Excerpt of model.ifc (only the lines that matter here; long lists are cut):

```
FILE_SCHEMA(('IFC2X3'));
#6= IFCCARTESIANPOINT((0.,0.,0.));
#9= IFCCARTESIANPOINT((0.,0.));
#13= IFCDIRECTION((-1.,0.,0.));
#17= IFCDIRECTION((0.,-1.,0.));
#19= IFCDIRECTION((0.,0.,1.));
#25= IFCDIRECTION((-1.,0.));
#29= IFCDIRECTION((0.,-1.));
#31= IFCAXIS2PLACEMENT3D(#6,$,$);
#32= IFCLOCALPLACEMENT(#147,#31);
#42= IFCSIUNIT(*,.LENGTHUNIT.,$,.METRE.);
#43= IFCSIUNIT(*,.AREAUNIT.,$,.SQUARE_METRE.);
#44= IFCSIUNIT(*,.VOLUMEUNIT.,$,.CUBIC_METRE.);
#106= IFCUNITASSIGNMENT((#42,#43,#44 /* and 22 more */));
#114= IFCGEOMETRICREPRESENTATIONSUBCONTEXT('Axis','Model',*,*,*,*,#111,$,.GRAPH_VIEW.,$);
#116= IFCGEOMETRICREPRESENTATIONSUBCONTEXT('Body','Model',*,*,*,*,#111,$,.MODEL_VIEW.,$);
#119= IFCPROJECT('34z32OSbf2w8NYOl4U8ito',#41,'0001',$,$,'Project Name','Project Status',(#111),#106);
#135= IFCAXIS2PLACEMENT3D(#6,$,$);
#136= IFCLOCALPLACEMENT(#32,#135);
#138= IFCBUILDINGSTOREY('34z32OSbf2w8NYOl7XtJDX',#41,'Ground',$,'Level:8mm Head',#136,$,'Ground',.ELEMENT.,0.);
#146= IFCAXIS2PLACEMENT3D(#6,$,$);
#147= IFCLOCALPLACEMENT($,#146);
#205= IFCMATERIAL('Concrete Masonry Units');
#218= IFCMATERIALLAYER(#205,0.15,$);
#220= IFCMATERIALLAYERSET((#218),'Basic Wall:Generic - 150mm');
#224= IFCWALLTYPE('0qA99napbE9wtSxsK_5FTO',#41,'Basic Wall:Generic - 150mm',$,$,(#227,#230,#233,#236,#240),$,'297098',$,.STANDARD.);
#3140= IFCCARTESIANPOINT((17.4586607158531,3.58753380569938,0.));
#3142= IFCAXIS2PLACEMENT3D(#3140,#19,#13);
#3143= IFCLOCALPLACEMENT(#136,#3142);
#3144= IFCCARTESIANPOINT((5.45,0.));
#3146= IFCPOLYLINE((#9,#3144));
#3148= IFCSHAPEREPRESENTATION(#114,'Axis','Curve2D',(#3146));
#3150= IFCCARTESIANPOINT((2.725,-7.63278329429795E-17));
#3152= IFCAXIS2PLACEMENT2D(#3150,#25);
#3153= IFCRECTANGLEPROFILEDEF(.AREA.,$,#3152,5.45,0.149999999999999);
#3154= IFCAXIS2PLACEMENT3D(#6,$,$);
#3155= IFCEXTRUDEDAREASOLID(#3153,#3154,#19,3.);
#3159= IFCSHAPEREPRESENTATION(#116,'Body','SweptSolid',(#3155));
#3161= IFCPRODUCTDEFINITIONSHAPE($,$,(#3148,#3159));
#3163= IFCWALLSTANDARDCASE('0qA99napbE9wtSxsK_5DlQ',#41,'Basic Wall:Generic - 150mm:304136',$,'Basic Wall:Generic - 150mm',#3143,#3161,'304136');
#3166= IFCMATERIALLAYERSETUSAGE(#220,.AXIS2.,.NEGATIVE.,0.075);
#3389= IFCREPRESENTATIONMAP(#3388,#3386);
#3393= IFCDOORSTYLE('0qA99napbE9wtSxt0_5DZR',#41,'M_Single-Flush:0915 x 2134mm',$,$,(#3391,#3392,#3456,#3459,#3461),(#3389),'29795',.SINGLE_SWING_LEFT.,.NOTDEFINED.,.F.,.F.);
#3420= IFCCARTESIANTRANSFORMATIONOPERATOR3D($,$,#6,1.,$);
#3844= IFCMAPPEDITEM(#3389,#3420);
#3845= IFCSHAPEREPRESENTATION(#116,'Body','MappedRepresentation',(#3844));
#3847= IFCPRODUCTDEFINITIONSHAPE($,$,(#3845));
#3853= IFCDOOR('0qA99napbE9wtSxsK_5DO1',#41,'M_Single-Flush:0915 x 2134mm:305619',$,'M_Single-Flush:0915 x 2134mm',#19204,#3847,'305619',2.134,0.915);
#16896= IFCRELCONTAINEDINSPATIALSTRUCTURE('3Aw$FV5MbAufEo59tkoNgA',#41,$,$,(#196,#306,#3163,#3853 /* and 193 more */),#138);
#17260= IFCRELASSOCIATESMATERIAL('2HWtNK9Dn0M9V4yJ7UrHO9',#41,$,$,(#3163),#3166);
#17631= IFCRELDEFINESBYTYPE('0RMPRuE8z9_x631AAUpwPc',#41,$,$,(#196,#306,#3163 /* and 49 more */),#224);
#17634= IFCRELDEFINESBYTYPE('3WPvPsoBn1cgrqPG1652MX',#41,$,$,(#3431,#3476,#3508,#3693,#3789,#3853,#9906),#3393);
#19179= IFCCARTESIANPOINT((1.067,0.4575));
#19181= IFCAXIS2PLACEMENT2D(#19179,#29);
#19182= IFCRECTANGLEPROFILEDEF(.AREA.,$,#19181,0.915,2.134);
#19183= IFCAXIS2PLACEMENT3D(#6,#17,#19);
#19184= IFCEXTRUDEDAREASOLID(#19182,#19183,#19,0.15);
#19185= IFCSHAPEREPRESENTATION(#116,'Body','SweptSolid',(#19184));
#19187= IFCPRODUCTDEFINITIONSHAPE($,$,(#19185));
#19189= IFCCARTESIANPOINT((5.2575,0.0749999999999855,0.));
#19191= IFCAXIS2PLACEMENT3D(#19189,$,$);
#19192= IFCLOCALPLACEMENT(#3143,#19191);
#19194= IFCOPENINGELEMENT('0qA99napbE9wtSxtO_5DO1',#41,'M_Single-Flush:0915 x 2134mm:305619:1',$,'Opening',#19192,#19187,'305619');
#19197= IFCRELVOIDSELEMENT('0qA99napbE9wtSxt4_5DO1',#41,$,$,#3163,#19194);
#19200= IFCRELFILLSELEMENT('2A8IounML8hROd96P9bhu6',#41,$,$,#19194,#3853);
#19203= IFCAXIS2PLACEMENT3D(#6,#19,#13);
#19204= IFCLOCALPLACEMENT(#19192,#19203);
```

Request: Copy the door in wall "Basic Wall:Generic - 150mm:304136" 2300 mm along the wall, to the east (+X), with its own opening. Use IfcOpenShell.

```python
import ifcopenshell
import ifcopenshell.api.feature
import ifcopenshell.api.geometry
import ifcopenshell.api.root
import ifcopenshell.geom
import ifcopenshell.util.element
import ifcopenshell.util.placement
import ifcopenshell.util.shape

model = ifcopenshell.open("model.ifc")
settings = ifcopenshell.geom.settings()


def volume(element):
    """Net volume in cubic metres, openings subtracted."""
    shape = ifcopenshell.geom.create_shape(settings, element)
    return ifcopenshell.util.shape.get_volume(shape.geometry)


def reuse_history(source, copy):
    """copy_class also copies each property set's owner history, people and application; keep the originals."""
    for rel in copy.IsDefinedBy:
        if rel.is_a("IfcRelDefinesByProperties") and (history := rel.RelatingPropertyDefinition.OwnerHistory):
            rel.RelatingPropertyDefinition.OwnerHistory = source.OwnerHistory
            ifcopenshell.util.element.remove_deep2(model, history)


door = model.by_guid("0qA99napbE9wtSxsK_5DO1")
opening = door.FillsVoids[0].RelatingOpeningElement
wall = opening.VoidsElements[0].RelatingBuildingElement
before = volume(wall)
shift = ifcopenshell.util.placement.get_local_placement(wall.ObjectPlacement)[:3, 0] * -2.3

# copy_class copies the void relationship, type, container and properties, but no geometry.
new_opening = ifcopenshell.api.root.copy_class(model, product=opening)
new_opening.Representation = ifcopenshell.util.element.copy_deep(
    model, opening.Representation, exclude=["IfcGeometricRepresentationContext", "IfcRepresentationMap"]
)
new_opening.Name = "M_Single-Flush:0915 x 2134mm"
new_opening.Tag = None
new_door = ifcopenshell.api.root.copy_class(model, product=door)
new_door.Representation = ifcopenshell.util.element.copy_deep(
    model, door.Representation, exclude=["IfcGeometricRepresentationContext", "IfcRepresentationMap"]
)
new_door.Name = "M_Single-Flush:0915 x 2134mm"
new_door.Tag = None
reuse_history(door, new_door)
fills = ifcopenshell.api.feature.add_filling(model, opening=new_opening, element=new_door)
fills.OwnerHistory = new_door.OwnerHistory  # required in IFC2X3

for old, new in ((opening, new_opening), (door, new_door)):
    matrix = ifcopenshell.util.placement.get_local_placement(old.ObjectPlacement)
    matrix[:3, 3] += shift
    ifcopenshell.api.geometry.edit_object_placement(model, product=new, matrix=matrix, is_si=False)

after = volume(wall)

print(f"wall volume {before:.3f} -> {after:.3f} m3")

model.write("model_v2.ifc")
```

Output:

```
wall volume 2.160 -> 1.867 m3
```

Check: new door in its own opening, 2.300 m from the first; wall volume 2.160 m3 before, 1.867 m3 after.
